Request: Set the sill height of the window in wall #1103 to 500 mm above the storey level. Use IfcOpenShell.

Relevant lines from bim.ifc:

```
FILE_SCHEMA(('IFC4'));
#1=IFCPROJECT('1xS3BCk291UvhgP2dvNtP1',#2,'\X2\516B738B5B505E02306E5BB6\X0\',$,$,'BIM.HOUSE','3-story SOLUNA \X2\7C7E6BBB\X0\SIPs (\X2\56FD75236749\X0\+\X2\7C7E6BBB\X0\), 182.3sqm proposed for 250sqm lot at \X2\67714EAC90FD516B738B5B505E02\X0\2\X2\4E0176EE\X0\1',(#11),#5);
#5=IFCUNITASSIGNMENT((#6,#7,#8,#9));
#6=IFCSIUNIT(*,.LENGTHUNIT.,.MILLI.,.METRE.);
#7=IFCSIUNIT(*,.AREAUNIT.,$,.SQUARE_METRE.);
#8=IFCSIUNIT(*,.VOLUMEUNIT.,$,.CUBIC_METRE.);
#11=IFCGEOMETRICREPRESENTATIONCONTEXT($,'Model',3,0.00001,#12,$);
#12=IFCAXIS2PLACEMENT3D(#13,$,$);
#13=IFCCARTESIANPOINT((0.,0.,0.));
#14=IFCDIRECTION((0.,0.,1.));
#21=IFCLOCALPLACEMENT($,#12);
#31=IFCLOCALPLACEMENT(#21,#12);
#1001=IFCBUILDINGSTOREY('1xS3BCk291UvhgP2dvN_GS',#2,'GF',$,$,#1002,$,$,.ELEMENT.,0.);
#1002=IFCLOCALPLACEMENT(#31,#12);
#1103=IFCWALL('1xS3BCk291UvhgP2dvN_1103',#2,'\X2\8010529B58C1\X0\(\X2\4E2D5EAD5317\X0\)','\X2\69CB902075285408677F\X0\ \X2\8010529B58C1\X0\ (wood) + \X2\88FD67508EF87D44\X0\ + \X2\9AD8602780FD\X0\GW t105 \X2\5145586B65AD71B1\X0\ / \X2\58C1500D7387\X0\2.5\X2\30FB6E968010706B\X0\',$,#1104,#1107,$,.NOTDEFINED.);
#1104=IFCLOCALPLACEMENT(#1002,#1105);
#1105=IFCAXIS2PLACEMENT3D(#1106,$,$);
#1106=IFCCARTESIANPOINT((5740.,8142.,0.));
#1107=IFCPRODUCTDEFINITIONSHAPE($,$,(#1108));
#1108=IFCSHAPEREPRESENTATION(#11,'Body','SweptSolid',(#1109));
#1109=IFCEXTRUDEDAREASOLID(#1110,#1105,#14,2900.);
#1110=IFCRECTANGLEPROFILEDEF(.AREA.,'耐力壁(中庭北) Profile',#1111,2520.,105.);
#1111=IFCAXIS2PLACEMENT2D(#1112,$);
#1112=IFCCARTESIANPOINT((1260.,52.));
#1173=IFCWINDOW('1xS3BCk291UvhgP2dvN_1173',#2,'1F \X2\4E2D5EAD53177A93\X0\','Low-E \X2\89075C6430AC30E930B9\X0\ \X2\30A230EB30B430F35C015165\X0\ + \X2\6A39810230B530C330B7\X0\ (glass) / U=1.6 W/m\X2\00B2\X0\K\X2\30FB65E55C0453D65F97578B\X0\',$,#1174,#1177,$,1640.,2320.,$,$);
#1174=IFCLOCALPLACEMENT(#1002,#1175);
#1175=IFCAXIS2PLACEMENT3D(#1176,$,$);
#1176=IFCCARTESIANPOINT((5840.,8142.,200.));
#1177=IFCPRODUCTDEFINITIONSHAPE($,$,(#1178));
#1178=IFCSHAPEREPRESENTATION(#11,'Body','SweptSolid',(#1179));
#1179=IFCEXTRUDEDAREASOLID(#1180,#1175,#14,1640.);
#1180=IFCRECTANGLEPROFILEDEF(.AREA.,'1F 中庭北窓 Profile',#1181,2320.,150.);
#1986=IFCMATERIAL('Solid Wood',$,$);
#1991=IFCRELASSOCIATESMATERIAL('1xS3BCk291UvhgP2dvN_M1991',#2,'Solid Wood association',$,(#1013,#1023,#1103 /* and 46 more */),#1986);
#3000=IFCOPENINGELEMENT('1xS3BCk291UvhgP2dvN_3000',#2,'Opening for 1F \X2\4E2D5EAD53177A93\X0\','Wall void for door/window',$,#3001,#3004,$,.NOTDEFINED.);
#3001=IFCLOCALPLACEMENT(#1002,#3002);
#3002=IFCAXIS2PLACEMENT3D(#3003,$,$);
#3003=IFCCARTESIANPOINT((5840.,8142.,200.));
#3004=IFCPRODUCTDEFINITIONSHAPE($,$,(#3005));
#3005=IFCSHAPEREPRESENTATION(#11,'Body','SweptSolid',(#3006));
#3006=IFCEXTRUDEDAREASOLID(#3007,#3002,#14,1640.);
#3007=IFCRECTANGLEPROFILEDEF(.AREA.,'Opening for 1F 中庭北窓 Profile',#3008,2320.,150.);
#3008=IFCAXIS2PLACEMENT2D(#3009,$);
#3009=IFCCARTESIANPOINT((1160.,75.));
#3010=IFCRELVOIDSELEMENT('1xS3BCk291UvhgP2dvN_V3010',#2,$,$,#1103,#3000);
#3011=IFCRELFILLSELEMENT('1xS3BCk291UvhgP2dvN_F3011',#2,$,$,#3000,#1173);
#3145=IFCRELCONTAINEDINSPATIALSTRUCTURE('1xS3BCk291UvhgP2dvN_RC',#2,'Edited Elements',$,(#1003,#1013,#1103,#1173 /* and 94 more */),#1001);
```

```python
import numpy as np
import ifcopenshell
import ifcopenshell.api.geometry
import ifcopenshell.geom
import ifcopenshell.util.element
import ifcopenshell.util.placement
import ifcopenshell.util.shape
import ifcopenshell.util.unit

model = ifcopenshell.open("bim.ifc")
unit_scale = ifcopenshell.util.unit.calculate_unit_scale(model)

window = model.by_id(1173)
opening = window.FillsVoids[0].RelatingOpeningElement
storey = ifcopenshell.util.element.get_container(window, ifc_class="IfcBuildingStorey")
level = ifcopenshell.util.placement.get_local_placement(storey.ObjectPlacement)[2, 3]

# The opening's origin need not be at the sill, so measure its lowest point.
shape = ifcopenshell.geom.create_shape(ifcopenshell.geom.settings(), opening)
bottom = ifcopenshell.util.shape.get_shape_bottom_elevation(shape, shape.geometry) / unit_scale
dz = level + 500.0 - bottom

shift = np.array([0.0, 0.0, dz])
# The window is not placed relative to its opening, so move both.
for product in (opening, window):
    matrix = ifcopenshell.util.placement.get_local_placement(product.ObjectPlacement)
    matrix[:3, 3] += shift
    ifcopenshell.api.geometry.edit_object_placement(model, product=product, matrix=matrix, is_si=False)

print(f"moved by {dz * unit_scale:+.3f} m")

model.write("bim-out.ifc")
```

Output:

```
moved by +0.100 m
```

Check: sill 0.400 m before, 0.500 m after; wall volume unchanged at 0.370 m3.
